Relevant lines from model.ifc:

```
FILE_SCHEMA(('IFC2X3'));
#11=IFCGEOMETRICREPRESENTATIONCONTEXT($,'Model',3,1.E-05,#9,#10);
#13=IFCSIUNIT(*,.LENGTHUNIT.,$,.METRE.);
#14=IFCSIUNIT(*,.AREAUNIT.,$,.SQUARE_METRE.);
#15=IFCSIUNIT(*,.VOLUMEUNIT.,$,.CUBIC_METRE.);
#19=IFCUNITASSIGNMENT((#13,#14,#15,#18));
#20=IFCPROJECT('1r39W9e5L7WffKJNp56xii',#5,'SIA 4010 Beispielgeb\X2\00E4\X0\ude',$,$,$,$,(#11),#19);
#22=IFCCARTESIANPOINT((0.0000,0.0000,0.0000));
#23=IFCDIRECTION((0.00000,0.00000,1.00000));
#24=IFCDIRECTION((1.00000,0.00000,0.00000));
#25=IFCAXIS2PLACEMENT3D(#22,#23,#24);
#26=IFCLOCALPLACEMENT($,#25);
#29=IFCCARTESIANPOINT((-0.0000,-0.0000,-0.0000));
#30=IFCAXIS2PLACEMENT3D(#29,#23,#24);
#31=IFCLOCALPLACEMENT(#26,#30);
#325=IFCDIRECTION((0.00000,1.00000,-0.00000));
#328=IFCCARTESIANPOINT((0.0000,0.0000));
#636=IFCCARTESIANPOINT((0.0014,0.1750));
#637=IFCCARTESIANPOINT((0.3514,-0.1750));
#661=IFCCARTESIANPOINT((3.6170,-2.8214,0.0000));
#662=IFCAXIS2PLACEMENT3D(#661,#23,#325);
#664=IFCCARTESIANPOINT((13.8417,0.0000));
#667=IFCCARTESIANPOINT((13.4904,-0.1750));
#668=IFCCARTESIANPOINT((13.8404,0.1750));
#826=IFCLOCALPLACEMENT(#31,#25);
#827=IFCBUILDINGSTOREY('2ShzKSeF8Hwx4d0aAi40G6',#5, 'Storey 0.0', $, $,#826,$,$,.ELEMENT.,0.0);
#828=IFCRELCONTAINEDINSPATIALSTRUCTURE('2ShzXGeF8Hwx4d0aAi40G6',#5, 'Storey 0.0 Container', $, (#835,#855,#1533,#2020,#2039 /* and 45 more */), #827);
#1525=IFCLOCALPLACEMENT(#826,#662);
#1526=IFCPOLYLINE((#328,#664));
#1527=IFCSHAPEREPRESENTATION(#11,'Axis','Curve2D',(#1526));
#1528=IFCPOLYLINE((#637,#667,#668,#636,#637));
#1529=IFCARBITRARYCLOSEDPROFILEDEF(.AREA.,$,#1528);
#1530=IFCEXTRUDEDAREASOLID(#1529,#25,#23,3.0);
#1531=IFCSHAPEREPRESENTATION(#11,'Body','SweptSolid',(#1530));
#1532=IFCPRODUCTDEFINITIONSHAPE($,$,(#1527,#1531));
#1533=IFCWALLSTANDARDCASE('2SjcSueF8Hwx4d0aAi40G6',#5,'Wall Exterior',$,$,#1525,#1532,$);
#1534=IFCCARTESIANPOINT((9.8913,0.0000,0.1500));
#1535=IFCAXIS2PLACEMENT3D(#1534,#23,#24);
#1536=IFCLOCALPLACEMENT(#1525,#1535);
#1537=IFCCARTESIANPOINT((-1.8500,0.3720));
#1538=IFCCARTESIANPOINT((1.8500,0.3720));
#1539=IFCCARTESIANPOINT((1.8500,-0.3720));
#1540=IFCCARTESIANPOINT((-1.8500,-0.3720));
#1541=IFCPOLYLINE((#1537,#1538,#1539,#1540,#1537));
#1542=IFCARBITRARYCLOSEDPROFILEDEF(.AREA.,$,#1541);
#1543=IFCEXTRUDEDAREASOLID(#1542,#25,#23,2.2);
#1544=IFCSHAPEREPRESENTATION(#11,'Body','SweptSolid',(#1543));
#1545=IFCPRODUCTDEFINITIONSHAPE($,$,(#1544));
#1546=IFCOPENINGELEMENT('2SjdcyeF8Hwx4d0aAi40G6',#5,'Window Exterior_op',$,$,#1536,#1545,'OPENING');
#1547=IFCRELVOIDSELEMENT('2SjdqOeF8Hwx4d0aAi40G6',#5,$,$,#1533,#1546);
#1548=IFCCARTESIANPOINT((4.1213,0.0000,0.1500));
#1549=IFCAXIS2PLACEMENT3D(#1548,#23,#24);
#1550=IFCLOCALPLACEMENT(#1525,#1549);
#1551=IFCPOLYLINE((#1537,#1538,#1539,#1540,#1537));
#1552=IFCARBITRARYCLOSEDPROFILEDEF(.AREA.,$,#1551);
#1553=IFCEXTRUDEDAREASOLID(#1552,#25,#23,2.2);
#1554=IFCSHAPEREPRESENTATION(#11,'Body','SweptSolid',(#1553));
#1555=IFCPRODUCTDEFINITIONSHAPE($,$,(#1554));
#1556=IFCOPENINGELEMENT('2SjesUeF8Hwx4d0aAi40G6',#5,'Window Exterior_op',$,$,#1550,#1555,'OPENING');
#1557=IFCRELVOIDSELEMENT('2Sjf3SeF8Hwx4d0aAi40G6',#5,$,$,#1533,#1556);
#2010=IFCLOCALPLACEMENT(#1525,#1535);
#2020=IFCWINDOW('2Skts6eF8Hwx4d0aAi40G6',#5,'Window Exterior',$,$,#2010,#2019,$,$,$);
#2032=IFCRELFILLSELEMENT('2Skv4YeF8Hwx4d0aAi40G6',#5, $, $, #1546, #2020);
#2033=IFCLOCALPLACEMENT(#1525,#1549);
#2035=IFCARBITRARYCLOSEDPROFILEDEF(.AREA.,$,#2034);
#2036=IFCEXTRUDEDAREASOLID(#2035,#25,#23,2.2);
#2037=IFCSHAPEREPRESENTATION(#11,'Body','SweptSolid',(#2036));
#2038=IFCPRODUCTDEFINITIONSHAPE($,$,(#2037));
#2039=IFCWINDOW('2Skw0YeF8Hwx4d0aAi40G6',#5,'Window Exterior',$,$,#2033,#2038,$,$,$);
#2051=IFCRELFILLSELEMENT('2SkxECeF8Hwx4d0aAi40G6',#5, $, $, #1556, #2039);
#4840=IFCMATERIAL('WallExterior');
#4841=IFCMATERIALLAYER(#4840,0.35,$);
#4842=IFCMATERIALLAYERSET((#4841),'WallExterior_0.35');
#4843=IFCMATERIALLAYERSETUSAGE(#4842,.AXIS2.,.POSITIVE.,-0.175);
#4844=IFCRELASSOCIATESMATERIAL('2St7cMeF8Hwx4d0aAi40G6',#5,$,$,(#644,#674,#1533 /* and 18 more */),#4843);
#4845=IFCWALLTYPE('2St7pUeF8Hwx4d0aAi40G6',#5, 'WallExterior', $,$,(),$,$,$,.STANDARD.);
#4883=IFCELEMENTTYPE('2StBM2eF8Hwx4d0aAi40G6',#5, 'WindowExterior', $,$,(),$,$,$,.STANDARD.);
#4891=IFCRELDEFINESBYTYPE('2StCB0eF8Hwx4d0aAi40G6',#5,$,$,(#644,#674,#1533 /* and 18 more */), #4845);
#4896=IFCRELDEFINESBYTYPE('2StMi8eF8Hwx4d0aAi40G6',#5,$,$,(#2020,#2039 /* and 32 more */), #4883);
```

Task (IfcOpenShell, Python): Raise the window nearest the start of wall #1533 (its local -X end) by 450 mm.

```python
import numpy as np
import ifcopenshell
import ifcopenshell.api.geometry
import ifcopenshell.util.placement
import ifcopenshell.util.unit

model = ifcopenshell.open("model.ifc")
unit_scale = ifcopenshell.util.unit.calculate_unit_scale(model)

window = model.by_guid("2Skw0YeF8Hwx4d0aAi40G6")
opening = window.FillsVoids[0].RelatingOpeningElement
dz = 0.45 / unit_scale

shift = np.array([0.0, 0.0, dz])
# The window is not placed relative to its opening, so move both.
for product in (opening, window):
    matrix = ifcopenshell.util.placement.get_local_placement(product.ObjectPlacement)
    matrix[:3, 3] += shift
    ifcopenshell.api.geometry.edit_object_placement(model, product=product, matrix=matrix, is_si=False)

print(f"moved by {dz * unit_scale:+.3f} m")

model.write("model_rev.ifc")
```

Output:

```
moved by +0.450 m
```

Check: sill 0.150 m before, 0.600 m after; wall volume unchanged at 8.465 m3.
